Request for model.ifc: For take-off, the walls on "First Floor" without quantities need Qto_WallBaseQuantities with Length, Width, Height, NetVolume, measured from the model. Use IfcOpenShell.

First a look at what the model holds.

```python
import ifcopenshell
import ifcopenshell.util.element
import ifcopenshell.util.unit

model = ifcopenshell.open("model.ifc")
print(model.schema)
for unit_type in ("LENGTHUNIT", "AREAUNIT", "VOLUMEUNIT"):
    print(unit_type, ifcopenshell.util.unit.calculate_unit_scale(model, unit_type))
storey = next(s for s in model.by_type("IfcBuildingStorey") if s.Name == "First Floor")
walls = [e for e in ifcopenshell.util.element.get_decomposition(storey) if e.is_a("IfcWall")]
for e in sorted(walls, key=lambda e: e.id()):
    print(e.id(), e.is_a(), e.Name, list(ifcopenshell.util.element.get_psets(e, qtos_only=True)), sep=" | ")
```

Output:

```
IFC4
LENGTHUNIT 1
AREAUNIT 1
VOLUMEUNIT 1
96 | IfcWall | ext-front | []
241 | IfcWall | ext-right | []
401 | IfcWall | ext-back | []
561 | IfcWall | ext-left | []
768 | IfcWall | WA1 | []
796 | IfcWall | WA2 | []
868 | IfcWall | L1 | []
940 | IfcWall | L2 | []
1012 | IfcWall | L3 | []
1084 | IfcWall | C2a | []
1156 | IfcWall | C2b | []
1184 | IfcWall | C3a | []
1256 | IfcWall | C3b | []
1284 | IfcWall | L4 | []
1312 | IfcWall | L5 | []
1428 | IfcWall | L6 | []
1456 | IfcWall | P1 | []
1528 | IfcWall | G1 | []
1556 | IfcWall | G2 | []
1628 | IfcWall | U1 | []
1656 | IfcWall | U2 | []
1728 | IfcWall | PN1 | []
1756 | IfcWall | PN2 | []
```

```python
import ifcopenshell
import ifcopenshell.api.pset
import ifcopenshell.geom
import ifcopenshell.util.element
import ifcopenshell.util.shape
import ifcopenshell.util.unit

model = ifcopenshell.open("model.ifc")
unit_scale = ifcopenshell.util.unit.calculate_unit_scale(model)
volume_scale = ifcopenshell.util.unit.calculate_unit_scale(model, "VOLUMEUNIT")
settings = ifcopenshell.geom.settings()

storey = next(s for s in model.by_type("IfcBuildingStorey") if s.Name == "First Floor")
walls = [e for e in ifcopenshell.util.element.get_decomposition(storey) if e.is_a("IfcWall")]

for e in sorted(walls, key=lambda e: e.id()):
    if ifcopenshell.util.element.get_psets(e, qtos_only=True, should_inherit=False):
        continue
    # Geometry comes back in metres, in the element's own axes.
    shape = ifcopenshell.geom.create_shape(settings, e)
    values = {
        "Length": ifcopenshell.util.shape.get_x(shape.geometry) / unit_scale,
        "Width": ifcopenshell.util.shape.get_y(shape.geometry) / unit_scale,
        "Height": ifcopenshell.util.shape.get_z(shape.geometry) / unit_scale,
        "NetVolume": ifcopenshell.util.shape.get_volume(shape.geometry) / volume_scale,
    }
    qto = ifcopenshell.api.pset.add_qto(model, product=e, name="Qto_WallBaseQuantities")
    ifcopenshell.api.pset.edit_qto(model, qto=qto, properties=values)
    print(e.id(), {k: round(v, 3) for k, v in values.items()})

model.write("model-out.ifc")
```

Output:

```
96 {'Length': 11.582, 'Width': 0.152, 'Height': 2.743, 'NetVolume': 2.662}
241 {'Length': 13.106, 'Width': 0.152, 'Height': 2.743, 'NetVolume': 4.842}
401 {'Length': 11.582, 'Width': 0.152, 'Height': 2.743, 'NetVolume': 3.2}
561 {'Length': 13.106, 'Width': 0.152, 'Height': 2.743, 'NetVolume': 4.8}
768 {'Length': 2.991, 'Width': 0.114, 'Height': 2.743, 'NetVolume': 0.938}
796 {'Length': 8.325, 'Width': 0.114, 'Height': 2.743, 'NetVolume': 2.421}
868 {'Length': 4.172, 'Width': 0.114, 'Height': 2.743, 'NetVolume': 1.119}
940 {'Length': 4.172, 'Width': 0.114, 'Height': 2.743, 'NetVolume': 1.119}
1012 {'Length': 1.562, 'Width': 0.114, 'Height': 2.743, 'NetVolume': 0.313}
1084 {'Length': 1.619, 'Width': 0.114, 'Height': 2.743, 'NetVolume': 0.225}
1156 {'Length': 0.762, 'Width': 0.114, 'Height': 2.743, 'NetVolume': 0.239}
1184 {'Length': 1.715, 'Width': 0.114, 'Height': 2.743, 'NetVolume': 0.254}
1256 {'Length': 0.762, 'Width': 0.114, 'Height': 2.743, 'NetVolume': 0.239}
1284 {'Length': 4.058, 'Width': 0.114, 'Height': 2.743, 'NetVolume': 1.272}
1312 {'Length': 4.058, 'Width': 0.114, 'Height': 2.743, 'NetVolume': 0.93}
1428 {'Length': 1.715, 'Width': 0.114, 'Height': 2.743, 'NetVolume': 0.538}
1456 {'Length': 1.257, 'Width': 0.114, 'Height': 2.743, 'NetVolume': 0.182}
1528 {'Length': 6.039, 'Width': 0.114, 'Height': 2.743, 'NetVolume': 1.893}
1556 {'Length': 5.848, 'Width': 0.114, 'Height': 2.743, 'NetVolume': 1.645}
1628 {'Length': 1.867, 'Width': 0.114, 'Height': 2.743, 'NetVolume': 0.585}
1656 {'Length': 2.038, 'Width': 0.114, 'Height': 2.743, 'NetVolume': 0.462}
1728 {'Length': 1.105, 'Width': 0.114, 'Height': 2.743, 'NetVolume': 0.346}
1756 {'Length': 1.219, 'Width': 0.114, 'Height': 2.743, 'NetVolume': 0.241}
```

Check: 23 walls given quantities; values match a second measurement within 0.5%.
